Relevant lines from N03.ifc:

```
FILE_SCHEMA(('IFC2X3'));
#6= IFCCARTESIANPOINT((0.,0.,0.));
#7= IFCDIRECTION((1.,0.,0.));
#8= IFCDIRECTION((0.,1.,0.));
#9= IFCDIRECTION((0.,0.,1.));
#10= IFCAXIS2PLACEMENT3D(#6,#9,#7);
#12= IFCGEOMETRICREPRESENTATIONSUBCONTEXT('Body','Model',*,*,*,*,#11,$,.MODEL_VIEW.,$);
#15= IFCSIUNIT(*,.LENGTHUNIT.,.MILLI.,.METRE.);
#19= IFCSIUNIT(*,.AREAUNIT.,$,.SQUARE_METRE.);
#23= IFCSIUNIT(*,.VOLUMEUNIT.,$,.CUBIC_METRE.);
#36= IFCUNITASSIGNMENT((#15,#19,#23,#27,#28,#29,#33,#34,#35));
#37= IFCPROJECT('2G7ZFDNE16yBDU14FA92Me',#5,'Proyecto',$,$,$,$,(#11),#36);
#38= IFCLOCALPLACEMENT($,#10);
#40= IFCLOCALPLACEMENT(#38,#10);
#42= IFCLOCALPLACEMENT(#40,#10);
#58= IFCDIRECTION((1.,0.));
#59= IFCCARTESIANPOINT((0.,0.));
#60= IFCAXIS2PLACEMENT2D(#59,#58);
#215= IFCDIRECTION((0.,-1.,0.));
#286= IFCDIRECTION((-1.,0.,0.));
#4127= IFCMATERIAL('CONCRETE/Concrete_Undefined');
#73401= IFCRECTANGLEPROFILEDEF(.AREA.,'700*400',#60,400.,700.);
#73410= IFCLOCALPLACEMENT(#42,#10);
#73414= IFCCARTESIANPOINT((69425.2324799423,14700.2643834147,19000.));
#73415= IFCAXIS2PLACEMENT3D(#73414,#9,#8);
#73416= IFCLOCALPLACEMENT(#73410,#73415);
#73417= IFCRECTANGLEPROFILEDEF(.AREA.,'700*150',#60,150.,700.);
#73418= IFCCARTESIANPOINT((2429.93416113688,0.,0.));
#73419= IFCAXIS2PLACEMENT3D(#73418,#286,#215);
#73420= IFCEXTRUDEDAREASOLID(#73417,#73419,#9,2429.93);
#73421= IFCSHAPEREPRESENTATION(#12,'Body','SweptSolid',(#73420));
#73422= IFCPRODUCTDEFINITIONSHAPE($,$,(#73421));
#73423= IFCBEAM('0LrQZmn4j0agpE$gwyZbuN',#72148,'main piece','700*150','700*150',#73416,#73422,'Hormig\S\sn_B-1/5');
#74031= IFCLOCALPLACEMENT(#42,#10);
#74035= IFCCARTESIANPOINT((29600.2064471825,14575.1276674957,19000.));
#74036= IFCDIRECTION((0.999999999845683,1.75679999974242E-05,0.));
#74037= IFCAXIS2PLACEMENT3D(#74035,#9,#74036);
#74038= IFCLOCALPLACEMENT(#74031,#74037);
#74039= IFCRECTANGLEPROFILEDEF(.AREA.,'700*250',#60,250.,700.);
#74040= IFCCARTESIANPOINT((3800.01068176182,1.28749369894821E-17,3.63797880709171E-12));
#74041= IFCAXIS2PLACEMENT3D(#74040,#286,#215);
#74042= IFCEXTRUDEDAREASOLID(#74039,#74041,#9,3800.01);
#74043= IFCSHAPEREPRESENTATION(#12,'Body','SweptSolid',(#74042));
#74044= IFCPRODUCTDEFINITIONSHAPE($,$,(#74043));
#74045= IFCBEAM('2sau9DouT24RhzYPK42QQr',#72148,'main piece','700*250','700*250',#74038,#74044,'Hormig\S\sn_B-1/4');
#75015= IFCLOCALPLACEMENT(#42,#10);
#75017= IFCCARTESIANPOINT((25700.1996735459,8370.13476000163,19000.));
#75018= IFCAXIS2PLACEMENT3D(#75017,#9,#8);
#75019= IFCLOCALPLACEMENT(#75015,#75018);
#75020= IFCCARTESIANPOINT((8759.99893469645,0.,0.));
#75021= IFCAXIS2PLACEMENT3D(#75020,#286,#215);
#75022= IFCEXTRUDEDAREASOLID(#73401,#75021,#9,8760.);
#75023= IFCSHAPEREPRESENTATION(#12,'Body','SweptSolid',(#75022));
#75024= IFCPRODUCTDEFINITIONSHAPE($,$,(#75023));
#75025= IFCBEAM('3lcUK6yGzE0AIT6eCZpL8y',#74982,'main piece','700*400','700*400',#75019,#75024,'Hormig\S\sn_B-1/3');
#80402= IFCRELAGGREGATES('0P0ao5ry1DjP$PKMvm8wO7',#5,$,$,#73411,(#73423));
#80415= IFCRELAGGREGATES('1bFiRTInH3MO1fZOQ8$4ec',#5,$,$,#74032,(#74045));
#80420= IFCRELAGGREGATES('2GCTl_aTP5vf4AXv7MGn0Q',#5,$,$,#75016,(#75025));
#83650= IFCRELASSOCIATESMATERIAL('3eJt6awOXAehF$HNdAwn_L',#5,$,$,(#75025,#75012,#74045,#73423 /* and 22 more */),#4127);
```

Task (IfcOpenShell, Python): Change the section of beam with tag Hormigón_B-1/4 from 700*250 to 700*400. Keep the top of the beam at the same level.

```python
import ifcopenshell
import ifcopenshell.util.element
import ifcopenshell.util.representation

model = ifcopenshell.open("N03.ifc")

member = model.by_guid("2sau9DouT24RhzYPK42QQr")
source = next(p for p in model.by_type("IfcRectangleProfileDef") if p.ProfileName == "700*400")

body = ifcopenshell.util.representation.get_representation(member, "Model", "Body")
solid = body.Items[0]
old_profile = solid.SweptArea

# Copy the section's sizes but keep this member's own profile position.
profile = ifcopenshell.util.element.copy(model, source)
# Profiles are centred, so shift by half the change in depth to hold the top.
shift = (old_profile.YDim - profile.YDim) / 2
x, y = old_profile.Position.Location.Coordinates
up = (0.0, 1.0)  # upwards, in the solid's own plane
location = model.createIfcCartesianPoint((x + up[0] * shift, y + up[1] * shift))
profile.Position = model.createIfcAxis2Placement2D(location, old_profile.Position.RefDirection)
solid.SweptArea = profile
if not model.get_total_inverses(old_profile):
    ifcopenshell.util.element.remove_deep2(model, old_profile)
member.Description = member.Description.replace("700*250", "700*400")
member.ObjectType = member.ObjectType.replace("700*250", "700*400")

print(solid.SweptArea)

model.write("N03_edited.ifc")
```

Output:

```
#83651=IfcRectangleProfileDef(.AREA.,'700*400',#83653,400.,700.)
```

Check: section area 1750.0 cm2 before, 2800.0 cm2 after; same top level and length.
